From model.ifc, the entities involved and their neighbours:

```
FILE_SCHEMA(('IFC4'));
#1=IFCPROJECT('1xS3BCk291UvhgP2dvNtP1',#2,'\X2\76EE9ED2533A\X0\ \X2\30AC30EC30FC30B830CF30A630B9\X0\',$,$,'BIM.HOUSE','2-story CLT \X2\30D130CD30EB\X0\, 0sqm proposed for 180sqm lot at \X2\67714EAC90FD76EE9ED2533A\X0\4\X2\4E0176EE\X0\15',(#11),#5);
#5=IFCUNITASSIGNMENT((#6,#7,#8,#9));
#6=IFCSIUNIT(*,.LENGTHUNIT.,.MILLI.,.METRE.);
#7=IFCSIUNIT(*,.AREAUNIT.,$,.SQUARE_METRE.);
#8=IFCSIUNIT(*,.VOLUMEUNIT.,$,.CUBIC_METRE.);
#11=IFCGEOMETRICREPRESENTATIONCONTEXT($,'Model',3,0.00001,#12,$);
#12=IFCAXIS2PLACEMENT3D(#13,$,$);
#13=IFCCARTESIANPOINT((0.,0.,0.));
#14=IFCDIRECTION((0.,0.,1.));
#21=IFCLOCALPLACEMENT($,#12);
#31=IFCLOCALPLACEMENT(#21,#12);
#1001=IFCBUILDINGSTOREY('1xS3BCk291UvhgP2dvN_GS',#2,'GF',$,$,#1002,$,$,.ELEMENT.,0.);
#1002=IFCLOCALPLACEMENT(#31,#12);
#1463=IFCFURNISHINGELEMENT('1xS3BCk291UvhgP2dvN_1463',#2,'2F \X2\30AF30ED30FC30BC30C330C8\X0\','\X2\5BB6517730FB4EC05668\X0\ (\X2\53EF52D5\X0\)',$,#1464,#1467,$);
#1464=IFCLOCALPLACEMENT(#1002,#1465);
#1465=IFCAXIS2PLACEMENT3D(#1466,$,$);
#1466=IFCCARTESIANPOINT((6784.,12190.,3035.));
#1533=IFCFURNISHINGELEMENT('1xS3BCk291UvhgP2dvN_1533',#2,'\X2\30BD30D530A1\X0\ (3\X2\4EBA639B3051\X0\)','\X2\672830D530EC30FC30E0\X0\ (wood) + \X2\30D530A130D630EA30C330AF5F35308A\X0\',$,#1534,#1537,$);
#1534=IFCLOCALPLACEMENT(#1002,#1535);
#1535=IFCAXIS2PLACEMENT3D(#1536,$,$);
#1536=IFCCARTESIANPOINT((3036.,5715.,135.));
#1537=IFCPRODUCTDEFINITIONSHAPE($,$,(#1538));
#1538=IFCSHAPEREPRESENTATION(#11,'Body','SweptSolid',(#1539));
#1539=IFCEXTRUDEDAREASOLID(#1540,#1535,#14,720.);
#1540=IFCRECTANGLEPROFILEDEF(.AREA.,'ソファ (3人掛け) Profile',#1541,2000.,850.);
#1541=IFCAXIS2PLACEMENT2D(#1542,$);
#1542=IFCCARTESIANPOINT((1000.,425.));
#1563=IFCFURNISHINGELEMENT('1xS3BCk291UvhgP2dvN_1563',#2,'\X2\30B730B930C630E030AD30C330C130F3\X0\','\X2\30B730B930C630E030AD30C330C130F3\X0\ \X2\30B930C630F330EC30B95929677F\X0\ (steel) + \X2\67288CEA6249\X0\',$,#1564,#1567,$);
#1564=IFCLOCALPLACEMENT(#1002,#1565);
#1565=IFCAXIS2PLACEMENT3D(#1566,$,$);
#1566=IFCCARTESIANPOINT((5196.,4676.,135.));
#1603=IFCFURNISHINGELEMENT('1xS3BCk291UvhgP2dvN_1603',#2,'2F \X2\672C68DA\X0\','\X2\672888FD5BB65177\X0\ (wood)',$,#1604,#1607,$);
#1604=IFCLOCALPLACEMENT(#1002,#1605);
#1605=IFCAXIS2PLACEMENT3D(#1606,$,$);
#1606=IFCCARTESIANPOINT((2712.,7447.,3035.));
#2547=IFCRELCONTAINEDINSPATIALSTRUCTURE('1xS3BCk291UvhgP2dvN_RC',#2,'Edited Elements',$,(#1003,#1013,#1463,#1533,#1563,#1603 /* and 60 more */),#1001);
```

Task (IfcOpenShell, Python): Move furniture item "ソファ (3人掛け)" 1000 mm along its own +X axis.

```python
import ifcopenshell
import ifcopenshell.api.geometry
import ifcopenshell.util.placement
import ifcopenshell.util.unit

model = ifcopenshell.open("model.ifc")
unit_scale = ifcopenshell.util.unit.calculate_unit_scale(model)

item = model.by_id(1533)
matrix = ifcopenshell.util.placement.get_local_placement(item.ObjectPlacement)
matrix[:3, 3] += matrix[:3, 0] * 1 / unit_scale
ifcopenshell.api.geometry.edit_object_placement(model, product=item, matrix=matrix, is_si=False)

print(ifcopenshell.util.placement.get_local_placement(item.ObjectPlacement).round(3) + 0.0)

model.write("model_v2.ifc")
```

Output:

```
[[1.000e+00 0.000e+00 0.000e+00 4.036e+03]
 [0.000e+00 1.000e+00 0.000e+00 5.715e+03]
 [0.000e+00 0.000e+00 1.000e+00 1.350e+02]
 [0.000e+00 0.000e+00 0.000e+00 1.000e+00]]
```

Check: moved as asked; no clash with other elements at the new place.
